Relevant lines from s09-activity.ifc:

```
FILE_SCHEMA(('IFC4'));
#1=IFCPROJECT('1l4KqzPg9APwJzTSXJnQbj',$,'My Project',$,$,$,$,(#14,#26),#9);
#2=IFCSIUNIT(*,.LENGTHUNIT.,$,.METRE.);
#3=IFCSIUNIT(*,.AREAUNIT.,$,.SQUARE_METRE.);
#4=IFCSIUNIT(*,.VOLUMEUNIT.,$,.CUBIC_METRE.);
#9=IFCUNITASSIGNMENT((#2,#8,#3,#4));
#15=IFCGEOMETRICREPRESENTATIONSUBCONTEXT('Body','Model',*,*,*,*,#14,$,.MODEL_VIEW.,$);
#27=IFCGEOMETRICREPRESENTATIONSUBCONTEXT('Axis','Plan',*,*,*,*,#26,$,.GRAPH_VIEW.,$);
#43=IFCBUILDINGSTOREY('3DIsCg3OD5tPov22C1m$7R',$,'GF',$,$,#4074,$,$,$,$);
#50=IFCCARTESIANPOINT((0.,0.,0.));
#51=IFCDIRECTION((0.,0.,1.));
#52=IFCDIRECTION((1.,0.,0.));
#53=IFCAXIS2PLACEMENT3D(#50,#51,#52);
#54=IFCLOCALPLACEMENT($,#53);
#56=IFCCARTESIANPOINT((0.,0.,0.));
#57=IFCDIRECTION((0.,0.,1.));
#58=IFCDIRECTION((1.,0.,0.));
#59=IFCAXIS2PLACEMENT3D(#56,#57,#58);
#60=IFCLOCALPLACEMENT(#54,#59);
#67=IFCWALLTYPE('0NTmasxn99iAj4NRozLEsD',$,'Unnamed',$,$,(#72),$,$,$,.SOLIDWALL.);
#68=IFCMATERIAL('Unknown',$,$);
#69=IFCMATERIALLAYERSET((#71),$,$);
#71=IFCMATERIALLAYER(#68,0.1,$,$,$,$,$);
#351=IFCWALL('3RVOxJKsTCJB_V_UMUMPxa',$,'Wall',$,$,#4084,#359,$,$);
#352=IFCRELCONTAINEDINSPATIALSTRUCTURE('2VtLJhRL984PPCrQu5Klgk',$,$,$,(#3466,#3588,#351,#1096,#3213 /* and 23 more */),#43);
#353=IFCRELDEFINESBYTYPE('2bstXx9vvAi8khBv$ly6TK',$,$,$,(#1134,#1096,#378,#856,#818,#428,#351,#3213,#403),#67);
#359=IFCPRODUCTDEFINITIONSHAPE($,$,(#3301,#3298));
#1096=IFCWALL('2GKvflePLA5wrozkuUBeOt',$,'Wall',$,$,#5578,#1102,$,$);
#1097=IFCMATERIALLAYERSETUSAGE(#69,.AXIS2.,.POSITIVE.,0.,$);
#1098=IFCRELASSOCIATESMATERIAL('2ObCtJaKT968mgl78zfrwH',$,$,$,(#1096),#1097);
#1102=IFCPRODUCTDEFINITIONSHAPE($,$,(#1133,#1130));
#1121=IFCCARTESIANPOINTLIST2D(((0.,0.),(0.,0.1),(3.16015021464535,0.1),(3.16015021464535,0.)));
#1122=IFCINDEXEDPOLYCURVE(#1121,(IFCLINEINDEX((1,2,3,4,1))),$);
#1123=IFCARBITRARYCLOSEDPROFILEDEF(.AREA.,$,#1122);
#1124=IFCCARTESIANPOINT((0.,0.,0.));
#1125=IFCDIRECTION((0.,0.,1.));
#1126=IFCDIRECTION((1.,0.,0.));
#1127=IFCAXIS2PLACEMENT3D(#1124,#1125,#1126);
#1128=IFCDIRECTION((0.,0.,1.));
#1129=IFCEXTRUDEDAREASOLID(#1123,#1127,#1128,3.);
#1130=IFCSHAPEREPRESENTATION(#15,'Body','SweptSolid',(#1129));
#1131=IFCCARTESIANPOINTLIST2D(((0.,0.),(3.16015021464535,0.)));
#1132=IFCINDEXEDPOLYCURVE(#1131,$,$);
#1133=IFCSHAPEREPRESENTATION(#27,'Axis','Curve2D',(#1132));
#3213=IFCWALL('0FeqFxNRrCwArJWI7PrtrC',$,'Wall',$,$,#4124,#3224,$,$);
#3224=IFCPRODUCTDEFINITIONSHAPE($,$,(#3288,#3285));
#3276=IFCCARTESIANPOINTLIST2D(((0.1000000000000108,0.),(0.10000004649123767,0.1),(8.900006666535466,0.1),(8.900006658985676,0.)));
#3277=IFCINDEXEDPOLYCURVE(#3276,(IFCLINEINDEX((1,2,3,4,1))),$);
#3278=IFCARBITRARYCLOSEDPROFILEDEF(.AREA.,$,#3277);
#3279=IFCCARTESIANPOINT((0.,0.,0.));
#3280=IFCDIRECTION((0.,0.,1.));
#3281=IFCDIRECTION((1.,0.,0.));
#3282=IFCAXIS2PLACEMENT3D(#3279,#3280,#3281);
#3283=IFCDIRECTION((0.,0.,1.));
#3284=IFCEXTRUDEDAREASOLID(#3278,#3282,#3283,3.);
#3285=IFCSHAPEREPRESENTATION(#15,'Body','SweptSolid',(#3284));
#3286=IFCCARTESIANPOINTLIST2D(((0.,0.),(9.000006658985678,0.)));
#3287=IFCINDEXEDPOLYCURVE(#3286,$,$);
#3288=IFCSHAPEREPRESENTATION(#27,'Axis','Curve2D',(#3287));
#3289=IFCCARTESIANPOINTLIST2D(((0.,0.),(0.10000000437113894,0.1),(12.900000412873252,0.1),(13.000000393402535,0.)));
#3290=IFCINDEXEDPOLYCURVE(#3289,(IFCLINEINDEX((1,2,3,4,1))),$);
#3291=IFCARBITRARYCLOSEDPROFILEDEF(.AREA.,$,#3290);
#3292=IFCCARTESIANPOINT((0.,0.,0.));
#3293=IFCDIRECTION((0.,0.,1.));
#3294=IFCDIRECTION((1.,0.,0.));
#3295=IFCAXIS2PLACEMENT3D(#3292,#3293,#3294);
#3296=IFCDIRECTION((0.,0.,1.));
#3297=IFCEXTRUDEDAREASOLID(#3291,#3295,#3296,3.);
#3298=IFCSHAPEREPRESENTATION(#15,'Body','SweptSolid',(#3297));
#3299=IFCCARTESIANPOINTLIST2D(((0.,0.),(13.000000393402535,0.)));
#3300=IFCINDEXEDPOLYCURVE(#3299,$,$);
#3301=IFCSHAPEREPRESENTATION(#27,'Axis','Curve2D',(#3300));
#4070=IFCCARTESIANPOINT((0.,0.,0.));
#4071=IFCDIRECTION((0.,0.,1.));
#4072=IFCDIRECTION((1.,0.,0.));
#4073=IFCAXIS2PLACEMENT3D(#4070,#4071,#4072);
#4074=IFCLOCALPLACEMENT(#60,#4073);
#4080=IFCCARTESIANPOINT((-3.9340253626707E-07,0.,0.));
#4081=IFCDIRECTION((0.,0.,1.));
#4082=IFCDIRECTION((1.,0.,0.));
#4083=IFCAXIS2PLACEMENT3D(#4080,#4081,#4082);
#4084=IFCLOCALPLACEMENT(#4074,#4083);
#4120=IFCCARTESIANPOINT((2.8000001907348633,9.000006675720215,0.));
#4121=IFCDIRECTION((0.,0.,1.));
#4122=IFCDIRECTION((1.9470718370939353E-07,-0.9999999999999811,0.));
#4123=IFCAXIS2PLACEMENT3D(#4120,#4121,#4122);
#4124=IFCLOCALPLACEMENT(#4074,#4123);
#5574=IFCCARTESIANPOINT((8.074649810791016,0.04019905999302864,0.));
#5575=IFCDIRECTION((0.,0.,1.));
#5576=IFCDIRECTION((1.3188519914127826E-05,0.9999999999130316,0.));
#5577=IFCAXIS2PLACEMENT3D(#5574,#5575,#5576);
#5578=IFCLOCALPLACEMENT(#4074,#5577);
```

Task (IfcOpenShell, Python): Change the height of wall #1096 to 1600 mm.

```python
import ifcopenshell
import ifcopenshell.geom
import ifcopenshell.util.representation
import ifcopenshell.util.shape

model = ifcopenshell.open("s09-activity.ifc")
settings = ifcopenshell.geom.settings()


def volume(element):
    """Net volume in cubic metres, openings subtracted."""
    shape = ifcopenshell.geom.create_shape(settings, element)
    return ifcopenshell.util.shape.get_volume(shape.geometry)


wall = model.by_guid("2GKvflePLA5wrozkuUBeOt")
before = volume(wall)

body = ifcopenshell.util.representation.get_representation(wall, "Model", "Body")
solid = body.Items[0]
old_height = solid.Depth
solid.Depth = 1.6
after = volume(wall)

print(f"height {old_height:g} -> {solid.Depth:g}, volume {before:.3f} -> {after:.3f} m3")

model.write("s09-activity-out.ifc")
```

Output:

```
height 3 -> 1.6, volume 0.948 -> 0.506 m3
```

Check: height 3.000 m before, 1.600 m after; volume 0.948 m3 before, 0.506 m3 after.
